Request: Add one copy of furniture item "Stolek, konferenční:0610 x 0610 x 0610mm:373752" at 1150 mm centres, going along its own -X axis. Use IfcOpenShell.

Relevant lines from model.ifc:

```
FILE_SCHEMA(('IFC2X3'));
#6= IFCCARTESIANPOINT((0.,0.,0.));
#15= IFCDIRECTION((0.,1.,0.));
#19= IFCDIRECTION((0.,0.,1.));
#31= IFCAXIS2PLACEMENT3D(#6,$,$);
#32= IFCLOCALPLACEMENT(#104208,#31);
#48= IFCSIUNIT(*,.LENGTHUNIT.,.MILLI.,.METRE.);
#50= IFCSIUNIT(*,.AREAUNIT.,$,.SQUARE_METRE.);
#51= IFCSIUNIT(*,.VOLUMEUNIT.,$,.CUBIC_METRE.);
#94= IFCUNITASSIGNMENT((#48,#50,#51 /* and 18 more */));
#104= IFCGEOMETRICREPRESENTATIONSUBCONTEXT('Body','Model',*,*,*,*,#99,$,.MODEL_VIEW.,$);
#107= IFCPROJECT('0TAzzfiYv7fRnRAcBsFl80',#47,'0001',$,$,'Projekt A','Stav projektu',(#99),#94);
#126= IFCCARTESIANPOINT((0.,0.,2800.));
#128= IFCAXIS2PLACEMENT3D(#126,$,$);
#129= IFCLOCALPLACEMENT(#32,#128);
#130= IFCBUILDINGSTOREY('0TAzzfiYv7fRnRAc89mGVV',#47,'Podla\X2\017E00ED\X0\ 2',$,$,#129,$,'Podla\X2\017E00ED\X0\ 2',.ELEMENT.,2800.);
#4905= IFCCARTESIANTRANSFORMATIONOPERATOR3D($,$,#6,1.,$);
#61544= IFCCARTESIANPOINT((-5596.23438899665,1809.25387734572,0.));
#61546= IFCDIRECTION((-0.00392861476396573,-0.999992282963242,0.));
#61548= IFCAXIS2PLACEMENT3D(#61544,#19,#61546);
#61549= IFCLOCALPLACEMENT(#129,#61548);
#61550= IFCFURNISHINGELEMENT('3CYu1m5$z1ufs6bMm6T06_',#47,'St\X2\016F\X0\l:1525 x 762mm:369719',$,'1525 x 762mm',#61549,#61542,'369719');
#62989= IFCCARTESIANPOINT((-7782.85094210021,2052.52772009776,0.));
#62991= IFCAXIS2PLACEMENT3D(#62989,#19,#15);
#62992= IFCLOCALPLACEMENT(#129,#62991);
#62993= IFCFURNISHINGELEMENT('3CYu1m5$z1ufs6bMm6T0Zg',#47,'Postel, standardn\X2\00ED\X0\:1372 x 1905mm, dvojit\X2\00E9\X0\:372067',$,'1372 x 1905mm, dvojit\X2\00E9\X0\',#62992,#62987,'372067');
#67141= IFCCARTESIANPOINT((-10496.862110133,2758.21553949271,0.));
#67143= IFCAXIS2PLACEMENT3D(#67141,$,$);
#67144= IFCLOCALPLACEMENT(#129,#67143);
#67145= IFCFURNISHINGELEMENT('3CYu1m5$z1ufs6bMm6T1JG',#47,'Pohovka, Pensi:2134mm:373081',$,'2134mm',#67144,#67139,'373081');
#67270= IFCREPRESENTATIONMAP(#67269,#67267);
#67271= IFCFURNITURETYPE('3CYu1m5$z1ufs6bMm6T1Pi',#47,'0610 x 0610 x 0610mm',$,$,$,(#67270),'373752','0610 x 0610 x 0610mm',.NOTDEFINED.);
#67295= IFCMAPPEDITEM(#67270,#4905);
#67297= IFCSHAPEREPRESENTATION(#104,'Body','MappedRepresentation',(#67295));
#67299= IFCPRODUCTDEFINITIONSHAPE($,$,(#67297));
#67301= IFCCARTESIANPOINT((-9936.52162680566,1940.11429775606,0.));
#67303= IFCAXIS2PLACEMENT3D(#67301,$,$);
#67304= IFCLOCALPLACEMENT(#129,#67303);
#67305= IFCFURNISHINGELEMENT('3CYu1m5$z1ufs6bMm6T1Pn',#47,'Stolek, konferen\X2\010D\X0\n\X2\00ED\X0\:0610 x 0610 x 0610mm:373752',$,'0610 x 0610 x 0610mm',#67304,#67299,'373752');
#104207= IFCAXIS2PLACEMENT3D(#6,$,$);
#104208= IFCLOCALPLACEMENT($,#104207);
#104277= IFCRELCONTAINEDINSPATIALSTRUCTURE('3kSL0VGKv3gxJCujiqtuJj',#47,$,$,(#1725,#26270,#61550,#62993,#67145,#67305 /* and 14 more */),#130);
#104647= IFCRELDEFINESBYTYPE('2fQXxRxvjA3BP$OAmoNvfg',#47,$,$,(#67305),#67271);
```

```python
import ifcopenshell
import ifcopenshell.api.geometry
import ifcopenshell.api.root
import ifcopenshell.util.element
import ifcopenshell.util.placement

model = ifcopenshell.open("model.ifc")

source = model.by_guid("3CYu1m5$z1ufs6bMm6T1Pn")
base = ifcopenshell.util.placement.get_local_placement(source.ObjectPlacement)
step = -base[:3, 0] * 1150.0

for i in range(1, 2):
    copy = ifcopenshell.api.root.copy_class(model, product=source)
    copy.Representation = ifcopenshell.util.element.copy_deep(
        model, source.Representation, exclude=["IfcGeometricRepresentationContext", "IfcRepresentationMap"]
    )
    copy.Name = "Stolek, konferenční:0610 x 0610 x 0610mm"
    copy.Tag = None
    matrix = base.copy()
    matrix[:3, 3] += i * step
    print("added at", matrix[:3, 3].round(3) + 0.0)
    ifcopenshell.api.geometry.edit_object_placement(model, product=copy, matrix=matrix, is_si=False)

model.write("model_v2.ifc")
```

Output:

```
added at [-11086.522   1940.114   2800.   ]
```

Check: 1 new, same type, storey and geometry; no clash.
